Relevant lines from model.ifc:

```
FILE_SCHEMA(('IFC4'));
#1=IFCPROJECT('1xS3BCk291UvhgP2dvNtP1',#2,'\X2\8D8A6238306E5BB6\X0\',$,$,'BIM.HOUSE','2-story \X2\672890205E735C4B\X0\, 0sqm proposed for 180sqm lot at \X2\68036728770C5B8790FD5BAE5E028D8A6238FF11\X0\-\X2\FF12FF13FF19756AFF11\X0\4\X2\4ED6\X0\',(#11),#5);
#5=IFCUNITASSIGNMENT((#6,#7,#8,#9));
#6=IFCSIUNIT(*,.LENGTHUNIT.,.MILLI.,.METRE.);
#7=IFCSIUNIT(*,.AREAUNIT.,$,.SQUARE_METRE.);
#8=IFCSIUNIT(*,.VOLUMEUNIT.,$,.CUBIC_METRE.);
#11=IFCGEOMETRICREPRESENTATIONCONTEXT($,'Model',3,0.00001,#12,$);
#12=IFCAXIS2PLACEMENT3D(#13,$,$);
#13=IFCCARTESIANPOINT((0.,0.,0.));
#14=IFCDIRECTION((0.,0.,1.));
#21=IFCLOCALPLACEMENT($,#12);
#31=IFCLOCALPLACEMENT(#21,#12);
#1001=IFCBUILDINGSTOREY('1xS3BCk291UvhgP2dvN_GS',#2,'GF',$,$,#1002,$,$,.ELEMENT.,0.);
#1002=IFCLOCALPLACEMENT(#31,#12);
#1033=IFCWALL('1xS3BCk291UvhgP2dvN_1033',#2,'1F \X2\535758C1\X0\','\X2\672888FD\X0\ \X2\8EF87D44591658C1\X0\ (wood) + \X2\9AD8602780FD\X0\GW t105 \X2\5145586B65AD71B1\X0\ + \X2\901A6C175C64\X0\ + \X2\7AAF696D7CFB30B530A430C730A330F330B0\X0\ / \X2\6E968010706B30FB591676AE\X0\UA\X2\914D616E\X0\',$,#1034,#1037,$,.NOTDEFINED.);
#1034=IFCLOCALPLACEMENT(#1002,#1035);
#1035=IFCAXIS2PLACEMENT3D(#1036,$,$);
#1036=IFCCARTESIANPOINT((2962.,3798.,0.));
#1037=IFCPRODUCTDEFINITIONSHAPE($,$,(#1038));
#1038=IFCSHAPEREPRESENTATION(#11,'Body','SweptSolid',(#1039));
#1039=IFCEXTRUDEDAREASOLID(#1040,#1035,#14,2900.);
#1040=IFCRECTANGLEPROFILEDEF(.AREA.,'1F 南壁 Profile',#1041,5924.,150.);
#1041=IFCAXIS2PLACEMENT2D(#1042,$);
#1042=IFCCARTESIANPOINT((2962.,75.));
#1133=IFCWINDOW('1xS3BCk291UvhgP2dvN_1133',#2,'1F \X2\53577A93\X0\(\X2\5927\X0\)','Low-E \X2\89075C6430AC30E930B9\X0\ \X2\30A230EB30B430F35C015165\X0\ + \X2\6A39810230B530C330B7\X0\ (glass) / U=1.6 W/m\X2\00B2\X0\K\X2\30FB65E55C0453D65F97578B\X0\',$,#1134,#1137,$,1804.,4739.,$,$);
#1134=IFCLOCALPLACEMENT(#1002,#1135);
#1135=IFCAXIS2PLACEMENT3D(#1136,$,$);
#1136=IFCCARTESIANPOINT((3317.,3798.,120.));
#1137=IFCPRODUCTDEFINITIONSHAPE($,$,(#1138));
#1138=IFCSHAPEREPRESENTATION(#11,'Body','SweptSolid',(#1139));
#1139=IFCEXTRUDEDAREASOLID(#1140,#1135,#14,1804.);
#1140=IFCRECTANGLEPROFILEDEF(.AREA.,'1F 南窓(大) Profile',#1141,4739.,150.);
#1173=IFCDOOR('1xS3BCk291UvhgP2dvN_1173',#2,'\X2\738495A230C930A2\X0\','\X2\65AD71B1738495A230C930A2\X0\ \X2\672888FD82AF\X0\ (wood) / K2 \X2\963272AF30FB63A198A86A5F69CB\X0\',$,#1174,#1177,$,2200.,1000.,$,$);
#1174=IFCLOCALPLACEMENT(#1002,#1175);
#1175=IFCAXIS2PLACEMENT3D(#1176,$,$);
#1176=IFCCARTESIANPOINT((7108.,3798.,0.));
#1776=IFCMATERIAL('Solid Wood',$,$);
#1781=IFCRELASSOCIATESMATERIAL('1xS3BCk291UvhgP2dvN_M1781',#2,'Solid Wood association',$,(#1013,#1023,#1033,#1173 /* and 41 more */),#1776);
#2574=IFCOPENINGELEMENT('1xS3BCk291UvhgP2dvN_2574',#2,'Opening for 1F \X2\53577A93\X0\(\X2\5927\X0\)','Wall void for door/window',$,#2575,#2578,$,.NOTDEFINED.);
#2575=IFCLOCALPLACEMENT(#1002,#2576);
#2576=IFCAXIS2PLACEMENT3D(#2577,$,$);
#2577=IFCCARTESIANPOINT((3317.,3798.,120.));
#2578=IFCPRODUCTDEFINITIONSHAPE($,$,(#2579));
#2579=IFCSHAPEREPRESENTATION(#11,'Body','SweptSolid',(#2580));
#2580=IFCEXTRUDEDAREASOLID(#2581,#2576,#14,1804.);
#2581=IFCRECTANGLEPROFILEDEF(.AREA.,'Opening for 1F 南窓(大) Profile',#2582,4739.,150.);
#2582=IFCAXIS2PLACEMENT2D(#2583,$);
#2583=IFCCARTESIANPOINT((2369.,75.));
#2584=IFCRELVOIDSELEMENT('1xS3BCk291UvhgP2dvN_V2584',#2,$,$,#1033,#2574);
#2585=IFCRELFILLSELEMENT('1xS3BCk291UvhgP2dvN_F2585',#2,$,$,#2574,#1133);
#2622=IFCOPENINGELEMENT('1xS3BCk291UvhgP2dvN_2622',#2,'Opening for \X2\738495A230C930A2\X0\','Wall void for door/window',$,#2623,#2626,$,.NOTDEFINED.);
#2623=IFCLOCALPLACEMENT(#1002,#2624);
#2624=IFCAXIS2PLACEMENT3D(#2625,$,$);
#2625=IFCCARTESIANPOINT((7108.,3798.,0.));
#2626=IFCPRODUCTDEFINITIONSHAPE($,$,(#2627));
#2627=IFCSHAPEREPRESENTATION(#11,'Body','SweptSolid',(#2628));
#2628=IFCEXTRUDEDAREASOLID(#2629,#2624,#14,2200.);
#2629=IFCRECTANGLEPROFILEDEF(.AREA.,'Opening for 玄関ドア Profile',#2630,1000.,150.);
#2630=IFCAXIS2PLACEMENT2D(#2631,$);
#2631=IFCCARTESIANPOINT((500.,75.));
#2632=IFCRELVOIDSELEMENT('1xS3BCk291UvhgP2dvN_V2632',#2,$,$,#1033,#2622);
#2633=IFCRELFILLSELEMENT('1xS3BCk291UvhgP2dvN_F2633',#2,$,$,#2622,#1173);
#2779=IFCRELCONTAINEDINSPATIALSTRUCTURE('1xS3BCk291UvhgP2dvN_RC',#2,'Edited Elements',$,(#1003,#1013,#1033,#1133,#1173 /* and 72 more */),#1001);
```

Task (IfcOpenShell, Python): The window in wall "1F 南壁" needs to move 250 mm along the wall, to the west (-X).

```python
import ifcopenshell
import ifcopenshell.api.geometry
import ifcopenshell.util.placement

model = ifcopenshell.open("model.ifc")

window = model.by_guid("1xS3BCk291UvhgP2dvN_1133")
opening = window.FillsVoids[0].RelatingOpeningElement
wall = opening.VoidsElements[0].RelatingBuildingElement

wall_matrix = ifcopenshell.util.placement.get_local_placement(wall.ObjectPlacement)
shift = wall_matrix[:3, 0] * -250.0
before = ifcopenshell.util.placement.get_local_placement(window.ObjectPlacement)[:3, 3].copy()

# The window is not placed relative to its opening, so move both.
for product in (opening, window):
    matrix = ifcopenshell.util.placement.get_local_placement(product.ObjectPlacement)
    matrix[:3, 3] += shift
    ifcopenshell.api.geometry.edit_object_placement(model, product=product, matrix=matrix, is_si=False)

after = ifcopenshell.util.placement.get_local_placement(window.ObjectPlacement)[:3, 3]
print("window moved by", (after - before).round(3) + 0.0)

model.write("model_rev.ifc")
```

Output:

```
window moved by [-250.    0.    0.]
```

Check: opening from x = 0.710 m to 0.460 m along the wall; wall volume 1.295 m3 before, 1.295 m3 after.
